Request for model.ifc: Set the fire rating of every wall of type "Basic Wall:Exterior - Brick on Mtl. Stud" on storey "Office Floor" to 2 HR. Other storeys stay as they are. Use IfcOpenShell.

First a look at what the model holds.

```python
import ifcopenshell
import ifcopenshell.util.element

model = ifcopenshell.open("model.ifc")
print(model.schema)
storey = next(s for s in model.by_type("IfcBuildingStorey") if s.Name == "Office Floor")
walls = [e for e in ifcopenshell.util.element.get_decomposition(storey) if e.is_a("IfcWall")]
seen = {}
for e in walls:
    element_type = ifcopenshell.util.element.get_type(e)
    key = (element_type.Name if element_type != e and element_type else None, ifcopenshell.util.element.get_pset(e, "Pset_WallCommon", "FireRating"))
    seen[key] = seen.get(key, 0) + 1
for (name, value), count in sorted(seen.items(), key=str):
    print(count, "x", name, "|", value)
```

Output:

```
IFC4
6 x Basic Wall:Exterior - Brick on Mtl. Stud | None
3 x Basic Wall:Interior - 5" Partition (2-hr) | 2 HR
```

```python
import ifcopenshell
import ifcopenshell.api.pset
import ifcopenshell.util.element

model = ifcopenshell.open("model.ifc")

storey = next(s for s in model.by_type("IfcBuildingStorey") if s.Name == "Office Floor")
walls = [e for e in ifcopenshell.util.element.get_decomposition(storey) if e.is_a("IfcWall")]

count = 0
for e in walls:
    element_type = ifcopenshell.util.element.get_type(e)
    if element_type in (None, e) or element_type.Name != "Basic Wall:Exterior - Brick on Mtl. Stud":
        continue
    # add_pset returns the element's existing set when there is one.
    pset = ifcopenshell.api.pset.add_pset(model, product=e, name="Pset_WallCommon")
    ifcopenshell.api.pset.edit_pset(model, pset=pset, properties={"FireRating": "2 HR"})
    count += 1

print(count, "walls updated")

model.write("model_v2.ifc")
```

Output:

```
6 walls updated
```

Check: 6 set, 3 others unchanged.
